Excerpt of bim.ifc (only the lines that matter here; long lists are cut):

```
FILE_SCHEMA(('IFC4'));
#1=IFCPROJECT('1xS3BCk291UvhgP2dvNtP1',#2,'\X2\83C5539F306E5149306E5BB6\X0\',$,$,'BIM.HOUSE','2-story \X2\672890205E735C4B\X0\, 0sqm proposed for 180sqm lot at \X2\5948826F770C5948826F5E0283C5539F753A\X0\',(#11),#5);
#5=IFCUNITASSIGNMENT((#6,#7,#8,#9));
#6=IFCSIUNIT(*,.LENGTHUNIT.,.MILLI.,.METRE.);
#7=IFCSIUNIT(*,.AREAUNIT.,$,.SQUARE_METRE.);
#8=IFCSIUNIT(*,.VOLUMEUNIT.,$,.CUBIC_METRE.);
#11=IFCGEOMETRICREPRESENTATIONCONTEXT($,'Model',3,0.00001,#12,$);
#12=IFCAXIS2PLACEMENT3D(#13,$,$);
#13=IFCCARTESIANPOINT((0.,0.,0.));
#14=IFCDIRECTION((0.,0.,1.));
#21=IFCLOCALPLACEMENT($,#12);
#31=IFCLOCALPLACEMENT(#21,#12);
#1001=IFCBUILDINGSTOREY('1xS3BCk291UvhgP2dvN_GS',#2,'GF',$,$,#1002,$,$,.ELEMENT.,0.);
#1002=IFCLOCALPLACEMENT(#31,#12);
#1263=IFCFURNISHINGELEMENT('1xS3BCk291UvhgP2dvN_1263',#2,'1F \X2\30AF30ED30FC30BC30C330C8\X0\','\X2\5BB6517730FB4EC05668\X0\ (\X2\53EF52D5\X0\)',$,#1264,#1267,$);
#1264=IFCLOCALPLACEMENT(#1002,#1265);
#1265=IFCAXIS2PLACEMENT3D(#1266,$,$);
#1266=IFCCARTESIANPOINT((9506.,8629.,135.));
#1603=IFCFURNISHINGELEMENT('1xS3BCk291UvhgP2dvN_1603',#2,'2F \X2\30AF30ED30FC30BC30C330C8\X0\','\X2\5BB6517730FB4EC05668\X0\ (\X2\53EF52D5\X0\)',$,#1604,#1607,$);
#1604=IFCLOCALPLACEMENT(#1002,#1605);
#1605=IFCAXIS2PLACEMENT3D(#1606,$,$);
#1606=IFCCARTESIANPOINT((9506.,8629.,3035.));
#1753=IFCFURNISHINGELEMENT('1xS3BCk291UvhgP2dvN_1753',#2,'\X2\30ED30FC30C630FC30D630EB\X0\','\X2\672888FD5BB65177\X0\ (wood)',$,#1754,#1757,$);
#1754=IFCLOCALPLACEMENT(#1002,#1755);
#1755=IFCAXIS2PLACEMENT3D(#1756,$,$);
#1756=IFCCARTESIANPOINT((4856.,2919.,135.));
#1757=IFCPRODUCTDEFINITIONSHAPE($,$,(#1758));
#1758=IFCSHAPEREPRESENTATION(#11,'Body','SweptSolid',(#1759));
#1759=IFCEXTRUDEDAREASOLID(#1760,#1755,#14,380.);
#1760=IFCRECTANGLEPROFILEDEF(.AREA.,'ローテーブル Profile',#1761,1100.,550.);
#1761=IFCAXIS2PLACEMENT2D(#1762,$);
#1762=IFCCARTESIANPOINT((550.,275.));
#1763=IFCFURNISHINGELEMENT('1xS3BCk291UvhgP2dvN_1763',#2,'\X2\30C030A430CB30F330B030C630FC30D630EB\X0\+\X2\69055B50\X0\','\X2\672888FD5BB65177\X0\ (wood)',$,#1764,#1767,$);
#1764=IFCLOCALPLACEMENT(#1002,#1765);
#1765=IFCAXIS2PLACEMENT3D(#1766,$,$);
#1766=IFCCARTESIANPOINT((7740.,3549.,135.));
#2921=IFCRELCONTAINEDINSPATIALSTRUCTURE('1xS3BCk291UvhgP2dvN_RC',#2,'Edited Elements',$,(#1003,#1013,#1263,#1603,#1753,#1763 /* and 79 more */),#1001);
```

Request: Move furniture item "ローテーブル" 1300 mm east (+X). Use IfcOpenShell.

```python
import ifcopenshell
import ifcopenshell.api.geometry
import ifcopenshell.util.placement

model = ifcopenshell.open("bim.ifc")

item = model.by_id(1753)
matrix = ifcopenshell.util.placement.get_local_placement(item.ObjectPlacement)
matrix[0, 3] += 1300.0
ifcopenshell.api.geometry.edit_object_placement(model, product=item, matrix=matrix, is_si=False)

print(ifcopenshell.util.placement.get_local_placement(item.ObjectPlacement).round(3) + 0.0)

model.write("bim_edited.ifc")
```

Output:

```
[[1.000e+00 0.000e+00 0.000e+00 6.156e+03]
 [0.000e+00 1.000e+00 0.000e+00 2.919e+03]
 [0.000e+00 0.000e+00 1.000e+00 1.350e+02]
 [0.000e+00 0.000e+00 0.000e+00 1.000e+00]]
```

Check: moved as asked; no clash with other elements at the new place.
